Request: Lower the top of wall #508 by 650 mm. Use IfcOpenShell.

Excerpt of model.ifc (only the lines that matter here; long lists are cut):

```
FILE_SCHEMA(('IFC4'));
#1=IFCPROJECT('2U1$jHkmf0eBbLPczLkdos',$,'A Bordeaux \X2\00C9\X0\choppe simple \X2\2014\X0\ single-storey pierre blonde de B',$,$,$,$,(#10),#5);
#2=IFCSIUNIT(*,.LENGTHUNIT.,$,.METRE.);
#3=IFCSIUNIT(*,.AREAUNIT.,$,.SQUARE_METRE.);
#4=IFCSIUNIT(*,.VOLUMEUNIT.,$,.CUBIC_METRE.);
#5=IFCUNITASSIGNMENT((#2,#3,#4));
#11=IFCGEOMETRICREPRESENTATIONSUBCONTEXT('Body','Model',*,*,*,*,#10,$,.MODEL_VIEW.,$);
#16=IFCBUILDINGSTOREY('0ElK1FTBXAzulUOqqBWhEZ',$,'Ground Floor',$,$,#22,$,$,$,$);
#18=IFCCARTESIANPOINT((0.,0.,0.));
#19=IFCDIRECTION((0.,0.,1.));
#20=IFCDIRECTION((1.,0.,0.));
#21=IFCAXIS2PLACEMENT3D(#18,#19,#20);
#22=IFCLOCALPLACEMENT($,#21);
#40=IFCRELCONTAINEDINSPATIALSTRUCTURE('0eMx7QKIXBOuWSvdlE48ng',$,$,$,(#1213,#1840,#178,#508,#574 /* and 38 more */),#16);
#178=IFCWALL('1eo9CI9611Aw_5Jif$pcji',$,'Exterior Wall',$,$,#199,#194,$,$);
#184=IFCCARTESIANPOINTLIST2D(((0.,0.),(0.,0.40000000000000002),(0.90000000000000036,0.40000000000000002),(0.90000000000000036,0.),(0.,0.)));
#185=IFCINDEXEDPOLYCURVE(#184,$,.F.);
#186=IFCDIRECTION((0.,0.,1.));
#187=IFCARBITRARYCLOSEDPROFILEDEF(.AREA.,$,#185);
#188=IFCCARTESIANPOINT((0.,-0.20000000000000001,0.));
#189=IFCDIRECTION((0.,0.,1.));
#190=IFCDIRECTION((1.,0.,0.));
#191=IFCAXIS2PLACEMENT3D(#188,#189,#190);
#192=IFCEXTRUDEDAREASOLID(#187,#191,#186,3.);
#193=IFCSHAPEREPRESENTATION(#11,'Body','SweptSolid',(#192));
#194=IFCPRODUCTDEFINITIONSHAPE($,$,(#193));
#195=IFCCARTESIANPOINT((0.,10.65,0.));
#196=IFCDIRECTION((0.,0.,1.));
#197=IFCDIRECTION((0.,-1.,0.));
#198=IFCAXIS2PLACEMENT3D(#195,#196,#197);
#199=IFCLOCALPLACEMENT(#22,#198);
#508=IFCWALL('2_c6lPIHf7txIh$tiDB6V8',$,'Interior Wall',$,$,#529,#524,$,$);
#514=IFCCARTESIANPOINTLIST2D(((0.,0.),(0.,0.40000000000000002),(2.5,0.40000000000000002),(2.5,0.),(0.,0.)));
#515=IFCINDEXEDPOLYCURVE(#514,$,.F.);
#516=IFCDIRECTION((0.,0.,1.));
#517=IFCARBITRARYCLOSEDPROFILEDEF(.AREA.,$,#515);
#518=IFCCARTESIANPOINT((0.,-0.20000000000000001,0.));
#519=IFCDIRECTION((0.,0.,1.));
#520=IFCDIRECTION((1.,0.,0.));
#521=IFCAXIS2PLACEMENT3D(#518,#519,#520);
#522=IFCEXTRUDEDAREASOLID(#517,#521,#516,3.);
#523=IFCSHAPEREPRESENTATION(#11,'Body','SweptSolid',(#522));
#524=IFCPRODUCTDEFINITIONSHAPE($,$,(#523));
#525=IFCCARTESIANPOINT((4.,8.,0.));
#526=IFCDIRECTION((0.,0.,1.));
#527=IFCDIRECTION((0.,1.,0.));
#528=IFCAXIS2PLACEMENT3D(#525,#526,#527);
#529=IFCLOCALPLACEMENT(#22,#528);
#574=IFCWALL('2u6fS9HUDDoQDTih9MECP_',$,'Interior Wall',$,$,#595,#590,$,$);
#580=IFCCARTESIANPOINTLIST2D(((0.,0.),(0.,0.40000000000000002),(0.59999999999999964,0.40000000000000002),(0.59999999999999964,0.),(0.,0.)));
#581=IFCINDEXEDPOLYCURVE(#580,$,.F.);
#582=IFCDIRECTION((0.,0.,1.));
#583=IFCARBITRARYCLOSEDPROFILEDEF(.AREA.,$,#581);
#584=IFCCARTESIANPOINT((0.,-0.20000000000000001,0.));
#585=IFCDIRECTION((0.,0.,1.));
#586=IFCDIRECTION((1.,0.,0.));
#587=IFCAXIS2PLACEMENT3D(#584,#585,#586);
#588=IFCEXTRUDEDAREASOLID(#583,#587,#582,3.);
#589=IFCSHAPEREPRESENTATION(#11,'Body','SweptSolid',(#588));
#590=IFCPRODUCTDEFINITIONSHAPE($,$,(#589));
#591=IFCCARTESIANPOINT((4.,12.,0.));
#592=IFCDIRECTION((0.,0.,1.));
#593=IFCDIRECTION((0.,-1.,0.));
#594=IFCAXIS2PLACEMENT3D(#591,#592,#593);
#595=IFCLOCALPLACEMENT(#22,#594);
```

```python
import ifcopenshell
import ifcopenshell.geom
import ifcopenshell.util.representation
import ifcopenshell.util.shape

model = ifcopenshell.open("model.ifc")
settings = ifcopenshell.geom.settings()


def volume(element):
    """Net volume in cubic metres, openings subtracted."""
    shape = ifcopenshell.geom.create_shape(settings, element)
    return ifcopenshell.util.shape.get_volume(shape.geometry)


wall = model.by_guid("2_c6lPIHf7txIh$tiDB6V8")
before = volume(wall)

body = ifcopenshell.util.representation.get_representation(wall, "Model", "Body")
solid = body.Items[0]
old_height = solid.Depth
solid.Depth -= 0.65
after = volume(wall)

print(f"height {old_height:g} -> {solid.Depth:g}, volume {before:.3f} -> {after:.3f} m3")

model.write("model-out.ifc")
```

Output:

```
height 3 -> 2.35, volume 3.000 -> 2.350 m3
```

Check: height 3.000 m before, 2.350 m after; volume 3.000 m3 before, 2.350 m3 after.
